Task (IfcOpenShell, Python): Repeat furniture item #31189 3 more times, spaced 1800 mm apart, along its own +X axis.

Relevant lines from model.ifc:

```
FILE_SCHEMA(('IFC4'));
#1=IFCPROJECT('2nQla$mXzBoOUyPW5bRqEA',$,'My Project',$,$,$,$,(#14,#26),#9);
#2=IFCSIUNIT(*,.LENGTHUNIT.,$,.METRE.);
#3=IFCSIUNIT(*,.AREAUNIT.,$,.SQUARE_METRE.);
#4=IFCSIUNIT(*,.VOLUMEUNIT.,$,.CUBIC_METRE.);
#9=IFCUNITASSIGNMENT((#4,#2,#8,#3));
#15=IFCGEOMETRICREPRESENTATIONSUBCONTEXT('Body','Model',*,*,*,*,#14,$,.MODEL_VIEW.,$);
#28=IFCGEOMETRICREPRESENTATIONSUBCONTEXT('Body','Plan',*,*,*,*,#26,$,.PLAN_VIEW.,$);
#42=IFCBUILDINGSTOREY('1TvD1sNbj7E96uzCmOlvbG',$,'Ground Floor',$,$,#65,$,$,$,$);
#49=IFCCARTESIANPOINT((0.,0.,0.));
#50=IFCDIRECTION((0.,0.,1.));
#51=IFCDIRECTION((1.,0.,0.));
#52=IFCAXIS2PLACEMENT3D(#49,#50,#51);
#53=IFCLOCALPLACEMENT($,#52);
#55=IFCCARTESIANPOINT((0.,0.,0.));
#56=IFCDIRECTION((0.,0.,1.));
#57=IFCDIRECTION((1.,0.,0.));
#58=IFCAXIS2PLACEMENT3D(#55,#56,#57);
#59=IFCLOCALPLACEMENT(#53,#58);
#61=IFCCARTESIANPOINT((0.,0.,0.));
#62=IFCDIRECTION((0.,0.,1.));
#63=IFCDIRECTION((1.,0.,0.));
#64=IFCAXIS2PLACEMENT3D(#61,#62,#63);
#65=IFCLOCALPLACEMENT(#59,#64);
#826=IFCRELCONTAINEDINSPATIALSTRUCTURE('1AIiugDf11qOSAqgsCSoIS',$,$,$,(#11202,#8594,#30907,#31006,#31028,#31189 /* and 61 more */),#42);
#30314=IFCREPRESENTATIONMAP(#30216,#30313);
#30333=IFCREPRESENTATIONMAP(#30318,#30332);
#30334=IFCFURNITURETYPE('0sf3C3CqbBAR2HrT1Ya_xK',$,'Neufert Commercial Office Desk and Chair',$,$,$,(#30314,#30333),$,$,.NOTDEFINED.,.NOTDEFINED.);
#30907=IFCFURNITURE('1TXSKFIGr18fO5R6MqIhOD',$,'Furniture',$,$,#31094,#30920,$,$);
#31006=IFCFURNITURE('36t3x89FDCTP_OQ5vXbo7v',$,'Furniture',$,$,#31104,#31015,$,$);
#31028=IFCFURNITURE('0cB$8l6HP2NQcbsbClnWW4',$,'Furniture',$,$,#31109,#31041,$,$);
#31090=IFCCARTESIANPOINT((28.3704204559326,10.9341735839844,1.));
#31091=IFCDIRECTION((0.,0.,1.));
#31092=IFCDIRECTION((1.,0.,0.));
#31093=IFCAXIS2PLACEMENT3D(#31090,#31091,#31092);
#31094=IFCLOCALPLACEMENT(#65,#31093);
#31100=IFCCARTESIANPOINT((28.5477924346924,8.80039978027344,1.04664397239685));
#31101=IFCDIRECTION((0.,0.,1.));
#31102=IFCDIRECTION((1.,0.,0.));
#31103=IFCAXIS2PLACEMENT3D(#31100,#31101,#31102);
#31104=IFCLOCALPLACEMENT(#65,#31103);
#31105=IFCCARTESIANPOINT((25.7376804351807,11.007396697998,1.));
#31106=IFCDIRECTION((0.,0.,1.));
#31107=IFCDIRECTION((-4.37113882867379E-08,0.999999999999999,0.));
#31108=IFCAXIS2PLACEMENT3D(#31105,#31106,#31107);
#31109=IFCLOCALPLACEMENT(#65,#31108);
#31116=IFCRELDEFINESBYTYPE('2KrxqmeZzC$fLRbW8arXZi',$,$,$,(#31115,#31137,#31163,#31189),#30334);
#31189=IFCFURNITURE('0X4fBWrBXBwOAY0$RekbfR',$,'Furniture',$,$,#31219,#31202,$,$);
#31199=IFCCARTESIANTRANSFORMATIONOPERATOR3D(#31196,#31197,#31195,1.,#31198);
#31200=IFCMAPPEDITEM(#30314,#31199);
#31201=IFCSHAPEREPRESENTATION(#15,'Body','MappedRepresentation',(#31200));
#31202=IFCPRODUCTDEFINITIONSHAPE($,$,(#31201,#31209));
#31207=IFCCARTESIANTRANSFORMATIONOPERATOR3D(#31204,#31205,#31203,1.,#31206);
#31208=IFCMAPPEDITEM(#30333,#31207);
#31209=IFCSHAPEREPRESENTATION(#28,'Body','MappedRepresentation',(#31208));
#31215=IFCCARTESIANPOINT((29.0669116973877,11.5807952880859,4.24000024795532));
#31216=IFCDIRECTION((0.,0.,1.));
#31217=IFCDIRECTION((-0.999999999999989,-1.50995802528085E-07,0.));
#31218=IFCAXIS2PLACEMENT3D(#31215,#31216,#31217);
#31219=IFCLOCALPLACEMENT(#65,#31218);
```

```python
import ifcopenshell
import ifcopenshell.api.geometry
import ifcopenshell.api.root
import ifcopenshell.util.element
import ifcopenshell.util.placement

model = ifcopenshell.open("model.ifc")

source = model.by_guid("0X4fBWrBXBwOAY0$RekbfR")
base = ifcopenshell.util.placement.get_local_placement(source.ObjectPlacement)
step = base[:3, 0] * 1.8

for i in range(1, 4):
    copy = ifcopenshell.api.root.copy_class(model, product=source)
    copy.Representation = ifcopenshell.util.element.copy_deep(
        model, source.Representation, exclude=["IfcGeometricRepresentationContext", "IfcRepresentationMap"]
    )
    matrix = base.copy()
    matrix[:3, 3] += i * step
    print("added at", matrix[:3, 3].round(3) + 0.0)
    ifcopenshell.api.geometry.edit_object_placement(model, product=copy, matrix=matrix, is_si=False)

model.write("model-out.ifc")
```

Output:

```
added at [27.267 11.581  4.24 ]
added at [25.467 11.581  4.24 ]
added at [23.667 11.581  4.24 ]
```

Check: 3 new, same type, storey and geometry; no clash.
